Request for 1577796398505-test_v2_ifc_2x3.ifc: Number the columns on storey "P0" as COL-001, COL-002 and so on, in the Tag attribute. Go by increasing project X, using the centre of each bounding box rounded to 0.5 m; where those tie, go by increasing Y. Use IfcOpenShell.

First a look at what the model holds.

```python
import ifcopenshell
import ifcopenshell.util.element
import ifcopenshell.util.placement

model = ifcopenshell.open("1577796398505-test_v2_ifc_2x3.ifc")
print(model.schema)
storey = next(s for s in model.by_type("IfcBuildingStorey") if s.Name == "P0")
columns = [e for e in ifcopenshell.util.element.get_decomposition(storey) if e.is_a("IfcColumn")]
for e in sorted(columns, key=lambda e: e.id()):
    origin = ifcopenshell.util.placement.get_local_placement(e.ObjectPlacement)[:3, 3]
    print(e.id(), e.Tag, e.Name, origin.round(2) + 0.0, sep=" | ")
```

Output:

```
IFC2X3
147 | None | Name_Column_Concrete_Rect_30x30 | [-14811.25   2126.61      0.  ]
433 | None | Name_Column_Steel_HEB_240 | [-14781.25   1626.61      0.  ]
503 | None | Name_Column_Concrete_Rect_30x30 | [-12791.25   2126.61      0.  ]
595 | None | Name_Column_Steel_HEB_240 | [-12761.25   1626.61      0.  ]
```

```python
import ifcopenshell
import ifcopenshell.geom
import ifcopenshell.util.element
import ifcopenshell.util.shape

model = ifcopenshell.open("1577796398505-test_v2_ifc_2x3.ifc")
settings = ifcopenshell.geom.settings()
settings.set("use-world-coords", True)


def centre(element):
    shape = ifcopenshell.geom.create_shape(settings, element)
    return ifcopenshell.util.shape.get_bbox_centroid(shape.geometry)


storey = next(s for s in model.by_type("IfcBuildingStorey") if s.Name == "P0")
columns = [e for e in ifcopenshell.util.element.get_decomposition(storey) if e.is_a("IfcColumn")]

# Insertion points can sit at a corner or the storey origin, so sort by the geometry (in metres).
centres = {e: centre(e) for e in columns}
columns.sort(key=lambda e: (round(centres[e][0] / 0.5), centres[e][1]))

for i, e in enumerate(columns, start=1):
    number = f"COL-0{i:02d}"
    e.Tag = number
    print(e.id(), number)

model.write("1577796398505-test_v2_ifc_2x3_rev.ifc")
```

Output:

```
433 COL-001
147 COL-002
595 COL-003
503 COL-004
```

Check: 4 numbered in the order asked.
